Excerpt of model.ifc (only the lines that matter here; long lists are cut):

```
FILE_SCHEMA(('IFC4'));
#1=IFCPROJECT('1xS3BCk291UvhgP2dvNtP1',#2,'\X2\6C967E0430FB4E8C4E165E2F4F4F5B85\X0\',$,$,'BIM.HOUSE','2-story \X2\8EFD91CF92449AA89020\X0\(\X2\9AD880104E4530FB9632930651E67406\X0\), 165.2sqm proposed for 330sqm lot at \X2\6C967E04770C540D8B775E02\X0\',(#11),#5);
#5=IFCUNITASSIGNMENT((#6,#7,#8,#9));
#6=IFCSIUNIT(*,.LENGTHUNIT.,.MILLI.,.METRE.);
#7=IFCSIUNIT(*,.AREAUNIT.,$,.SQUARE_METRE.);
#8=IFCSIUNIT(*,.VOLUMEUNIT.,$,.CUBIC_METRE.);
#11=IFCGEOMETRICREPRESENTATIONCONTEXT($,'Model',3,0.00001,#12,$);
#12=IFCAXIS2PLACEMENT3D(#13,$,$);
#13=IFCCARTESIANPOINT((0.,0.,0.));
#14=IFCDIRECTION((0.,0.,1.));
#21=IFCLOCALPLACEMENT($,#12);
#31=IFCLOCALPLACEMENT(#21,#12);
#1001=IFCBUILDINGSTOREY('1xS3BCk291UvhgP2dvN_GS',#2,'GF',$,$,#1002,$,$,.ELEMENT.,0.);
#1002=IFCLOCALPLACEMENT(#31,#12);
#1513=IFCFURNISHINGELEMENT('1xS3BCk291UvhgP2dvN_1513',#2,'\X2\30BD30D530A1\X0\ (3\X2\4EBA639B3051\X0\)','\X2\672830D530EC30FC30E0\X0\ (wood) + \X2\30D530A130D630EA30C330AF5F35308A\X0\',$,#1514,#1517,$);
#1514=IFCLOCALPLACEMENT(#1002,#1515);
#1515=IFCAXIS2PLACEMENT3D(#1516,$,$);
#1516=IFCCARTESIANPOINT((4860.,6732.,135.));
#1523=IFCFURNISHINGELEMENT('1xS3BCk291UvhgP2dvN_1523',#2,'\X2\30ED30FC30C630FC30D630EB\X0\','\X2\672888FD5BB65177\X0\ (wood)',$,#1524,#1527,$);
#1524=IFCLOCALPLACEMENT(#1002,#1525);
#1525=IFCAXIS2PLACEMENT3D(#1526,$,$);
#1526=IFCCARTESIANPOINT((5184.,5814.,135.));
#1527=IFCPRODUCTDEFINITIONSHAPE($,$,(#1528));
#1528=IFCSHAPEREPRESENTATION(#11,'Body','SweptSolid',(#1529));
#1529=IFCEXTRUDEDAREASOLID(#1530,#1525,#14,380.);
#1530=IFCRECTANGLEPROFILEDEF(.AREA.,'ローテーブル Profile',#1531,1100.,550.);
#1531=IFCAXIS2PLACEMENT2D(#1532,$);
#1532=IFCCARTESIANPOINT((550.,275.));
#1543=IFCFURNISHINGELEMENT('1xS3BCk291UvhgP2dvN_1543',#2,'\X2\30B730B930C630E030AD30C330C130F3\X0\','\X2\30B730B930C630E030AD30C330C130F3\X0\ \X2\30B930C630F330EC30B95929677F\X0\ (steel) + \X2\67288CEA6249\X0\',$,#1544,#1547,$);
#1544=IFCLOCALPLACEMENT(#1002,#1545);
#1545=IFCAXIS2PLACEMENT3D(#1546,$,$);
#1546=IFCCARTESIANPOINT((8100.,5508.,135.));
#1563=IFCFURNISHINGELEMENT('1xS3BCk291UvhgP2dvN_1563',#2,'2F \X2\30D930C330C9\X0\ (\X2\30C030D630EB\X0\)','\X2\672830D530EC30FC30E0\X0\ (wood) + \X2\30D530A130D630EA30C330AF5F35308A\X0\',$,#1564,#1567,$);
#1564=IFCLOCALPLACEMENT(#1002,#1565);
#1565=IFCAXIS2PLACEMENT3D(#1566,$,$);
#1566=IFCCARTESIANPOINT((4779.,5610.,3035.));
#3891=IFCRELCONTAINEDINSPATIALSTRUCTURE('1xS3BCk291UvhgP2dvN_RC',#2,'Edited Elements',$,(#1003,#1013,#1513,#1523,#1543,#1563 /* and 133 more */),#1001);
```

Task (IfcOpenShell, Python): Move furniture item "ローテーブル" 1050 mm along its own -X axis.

```python
import ifcopenshell
import ifcopenshell.api.geometry
import ifcopenshell.util.placement
import ifcopenshell.util.unit

model = ifcopenshell.open("model.ifc")
unit_scale = ifcopenshell.util.unit.calculate_unit_scale(model)

item = model.by_guid("1xS3BCk291UvhgP2dvN_1523")
matrix = ifcopenshell.util.placement.get_local_placement(item.ObjectPlacement)
matrix[:3, 3] -= matrix[:3, 0] * 1.05 / unit_scale
ifcopenshell.api.geometry.edit_object_placement(model, product=item, matrix=matrix, is_si=False)

print(ifcopenshell.util.placement.get_local_placement(item.ObjectPlacement).round(3) + 0.0)

model.write("model_edited.ifc")
```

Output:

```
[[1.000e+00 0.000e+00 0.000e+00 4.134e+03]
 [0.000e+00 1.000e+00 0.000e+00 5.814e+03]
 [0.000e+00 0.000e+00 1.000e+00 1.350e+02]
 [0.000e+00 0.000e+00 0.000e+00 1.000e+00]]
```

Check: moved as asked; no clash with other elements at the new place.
